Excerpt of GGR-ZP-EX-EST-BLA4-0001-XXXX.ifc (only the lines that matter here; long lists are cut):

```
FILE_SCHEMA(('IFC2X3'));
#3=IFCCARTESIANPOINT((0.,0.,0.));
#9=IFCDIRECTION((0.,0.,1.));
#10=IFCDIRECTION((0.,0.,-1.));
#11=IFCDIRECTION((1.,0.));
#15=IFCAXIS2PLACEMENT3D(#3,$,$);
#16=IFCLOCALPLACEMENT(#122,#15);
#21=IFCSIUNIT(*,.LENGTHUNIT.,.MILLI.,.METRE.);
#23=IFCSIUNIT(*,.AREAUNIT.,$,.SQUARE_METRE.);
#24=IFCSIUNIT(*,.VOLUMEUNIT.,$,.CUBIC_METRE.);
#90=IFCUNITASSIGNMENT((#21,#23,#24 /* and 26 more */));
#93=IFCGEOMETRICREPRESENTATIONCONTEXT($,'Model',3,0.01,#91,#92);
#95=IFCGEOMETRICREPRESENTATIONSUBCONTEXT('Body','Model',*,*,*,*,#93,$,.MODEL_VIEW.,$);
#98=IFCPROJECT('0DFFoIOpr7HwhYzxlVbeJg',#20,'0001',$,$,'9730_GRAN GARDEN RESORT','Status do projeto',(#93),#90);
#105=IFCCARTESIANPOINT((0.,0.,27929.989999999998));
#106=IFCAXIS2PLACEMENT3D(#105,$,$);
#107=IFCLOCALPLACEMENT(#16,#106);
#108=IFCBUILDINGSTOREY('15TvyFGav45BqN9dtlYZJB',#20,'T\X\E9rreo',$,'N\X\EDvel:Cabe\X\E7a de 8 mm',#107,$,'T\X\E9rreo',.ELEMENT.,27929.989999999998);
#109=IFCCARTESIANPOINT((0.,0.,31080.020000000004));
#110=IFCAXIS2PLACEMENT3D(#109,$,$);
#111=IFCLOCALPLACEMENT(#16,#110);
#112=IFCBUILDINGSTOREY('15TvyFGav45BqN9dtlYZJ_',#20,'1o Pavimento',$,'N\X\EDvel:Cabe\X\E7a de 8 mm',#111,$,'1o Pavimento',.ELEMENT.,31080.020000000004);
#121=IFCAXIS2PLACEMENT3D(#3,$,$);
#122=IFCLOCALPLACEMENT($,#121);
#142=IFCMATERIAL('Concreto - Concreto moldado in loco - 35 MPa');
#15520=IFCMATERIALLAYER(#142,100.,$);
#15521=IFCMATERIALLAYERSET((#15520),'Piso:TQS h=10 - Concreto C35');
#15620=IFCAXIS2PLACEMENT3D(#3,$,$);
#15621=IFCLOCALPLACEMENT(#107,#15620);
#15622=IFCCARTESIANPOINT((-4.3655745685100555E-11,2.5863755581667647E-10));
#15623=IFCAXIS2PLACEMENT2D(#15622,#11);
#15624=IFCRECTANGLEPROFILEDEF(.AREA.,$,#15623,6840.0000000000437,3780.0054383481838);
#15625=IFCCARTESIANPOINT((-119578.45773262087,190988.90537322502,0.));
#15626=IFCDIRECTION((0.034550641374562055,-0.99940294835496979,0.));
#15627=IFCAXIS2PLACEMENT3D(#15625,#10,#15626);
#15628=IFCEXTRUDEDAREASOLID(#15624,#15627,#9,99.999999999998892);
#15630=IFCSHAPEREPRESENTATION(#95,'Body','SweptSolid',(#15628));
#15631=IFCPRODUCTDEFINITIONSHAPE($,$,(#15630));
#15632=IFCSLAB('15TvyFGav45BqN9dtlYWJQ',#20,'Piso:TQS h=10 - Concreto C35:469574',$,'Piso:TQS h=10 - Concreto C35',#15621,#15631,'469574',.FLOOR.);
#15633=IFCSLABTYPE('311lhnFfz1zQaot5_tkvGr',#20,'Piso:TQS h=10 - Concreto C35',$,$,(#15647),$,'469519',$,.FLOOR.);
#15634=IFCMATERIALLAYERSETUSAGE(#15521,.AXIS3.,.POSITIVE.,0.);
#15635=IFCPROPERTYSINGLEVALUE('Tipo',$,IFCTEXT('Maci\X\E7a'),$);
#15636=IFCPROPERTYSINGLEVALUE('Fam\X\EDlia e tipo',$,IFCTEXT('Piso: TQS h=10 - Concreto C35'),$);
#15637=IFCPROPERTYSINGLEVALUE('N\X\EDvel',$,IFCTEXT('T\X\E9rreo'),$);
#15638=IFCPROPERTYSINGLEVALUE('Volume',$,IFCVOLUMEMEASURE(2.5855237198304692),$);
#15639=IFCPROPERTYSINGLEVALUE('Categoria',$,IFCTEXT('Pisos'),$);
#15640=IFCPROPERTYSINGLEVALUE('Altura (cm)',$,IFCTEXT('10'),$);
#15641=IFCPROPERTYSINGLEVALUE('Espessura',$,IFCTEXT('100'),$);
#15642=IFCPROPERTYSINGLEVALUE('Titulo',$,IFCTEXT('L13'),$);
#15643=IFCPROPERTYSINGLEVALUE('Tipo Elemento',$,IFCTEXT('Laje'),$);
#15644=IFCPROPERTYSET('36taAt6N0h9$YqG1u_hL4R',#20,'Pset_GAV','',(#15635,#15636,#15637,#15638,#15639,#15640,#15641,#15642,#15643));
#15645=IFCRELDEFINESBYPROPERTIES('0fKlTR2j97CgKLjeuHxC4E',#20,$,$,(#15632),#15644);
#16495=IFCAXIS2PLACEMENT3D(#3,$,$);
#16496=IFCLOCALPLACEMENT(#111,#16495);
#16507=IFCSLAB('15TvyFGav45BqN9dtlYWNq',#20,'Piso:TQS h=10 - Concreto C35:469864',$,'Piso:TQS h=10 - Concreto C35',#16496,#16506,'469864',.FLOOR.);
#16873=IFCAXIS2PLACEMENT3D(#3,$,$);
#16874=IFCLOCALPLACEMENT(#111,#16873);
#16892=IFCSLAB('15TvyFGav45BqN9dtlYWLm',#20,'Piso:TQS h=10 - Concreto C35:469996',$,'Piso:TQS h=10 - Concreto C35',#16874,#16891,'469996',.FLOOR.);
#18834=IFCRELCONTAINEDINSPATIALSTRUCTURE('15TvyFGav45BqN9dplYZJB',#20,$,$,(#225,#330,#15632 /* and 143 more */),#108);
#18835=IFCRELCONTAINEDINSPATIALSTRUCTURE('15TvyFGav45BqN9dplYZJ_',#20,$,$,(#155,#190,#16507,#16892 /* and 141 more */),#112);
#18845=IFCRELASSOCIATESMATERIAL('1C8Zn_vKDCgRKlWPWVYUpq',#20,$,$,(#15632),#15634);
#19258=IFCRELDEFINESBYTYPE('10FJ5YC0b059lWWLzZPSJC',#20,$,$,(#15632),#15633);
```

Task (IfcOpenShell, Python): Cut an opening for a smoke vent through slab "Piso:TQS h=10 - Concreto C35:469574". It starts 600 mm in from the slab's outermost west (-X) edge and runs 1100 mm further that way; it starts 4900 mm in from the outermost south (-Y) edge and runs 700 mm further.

```python
import numpy as np
import ifcopenshell
import ifcopenshell.api.feature
import ifcopenshell.api.geometry
import ifcopenshell.api.pset
import ifcopenshell.api.root
import ifcopenshell.geom
import ifcopenshell.util.element
import ifcopenshell.util.placement
import ifcopenshell.util.representation
import ifcopenshell.util.shape
import ifcopenshell.util.unit

model = ifcopenshell.open("GGR-ZP-EX-EST-BLA4-0001-XXXX.ifc")
unit_scale = ifcopenshell.util.unit.calculate_unit_scale(model)
volume_scale = ifcopenshell.util.unit.calculate_unit_scale(model, "VOLUMEUNIT")
settings = ifcopenshell.geom.settings()


def volume(element):
    """Net volume in cubic metres, openings subtracted."""
    shape = ifcopenshell.geom.create_shape(settings, element)
    return ifcopenshell.util.shape.get_volume(shape.geometry)


slab = model.by_guid("15TvyFGav45BqN9dtlYWJQ")
before = volume(slab)

# Extent in the slab's own axes, in metres. The edges named are its -X and -Y sides.
slab_shape = ifcopenshell.geom.create_shape(settings, slab)
vertices = ifcopenshell.util.shape.get_vertices(slab_shape.geometry)
x_min, y_min, bottom = vertices.min(axis=0)
top = vertices[:, 2].max()

opening = ifcopenshell.api.root.create_entity(model, ifc_class="IfcOpeningElement", name="Smoke vent opening")
context = ifcopenshell.util.representation.get_context(model, "Model", "Body", "MODEL_VIEW")
width, depth = 1.1, 0.7
outline = [(0.0, 0.0), (width, 0.0), (width, depth), (0.0, depth), (0.0, 0.0)]
# Overshoot both faces by 50 mm so the cut is clean.
shape = ifcopenshell.api.geometry.add_slab_representation(
    model, context=context, depth=top - bottom + 0.1, polyline=outline
)
ifcopenshell.api.geometry.assign_representation(model, product=opening, representation=shape)

matrix = ifcopenshell.util.placement.get_local_placement(slab.ObjectPlacement)
matrix[:, 3] = matrix @ np.append(np.array([x_min + 0.6, y_min + 4.9, bottom - 0.05]) / unit_scale, 1.0)
ifcopenshell.api.geometry.edit_object_placement(model, product=opening, matrix=matrix, is_si=False)
ifcopenshell.api.feature.add_feature(model, feature=opening, element=slab)

after = volume(slab)

# Update the slab's stored quantities.
pset = model.by_id(ifcopenshell.util.element.get_pset(slab, "Pset_GAV", should_inherit=False)["id"])
ifcopenshell.api.pset.edit_pset(model, pset=pset, properties={
    "Volume": model.create_entity("IfcVolumeMeasure", after / volume_scale),
})

print(f"slab volume {before:.3f} -> {after:.3f} m3")

model.write("GGR-ZP-EX-EST-BLA4-0001-XXXX-out.ifc")
```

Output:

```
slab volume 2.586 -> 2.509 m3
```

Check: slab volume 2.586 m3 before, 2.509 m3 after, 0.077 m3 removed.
